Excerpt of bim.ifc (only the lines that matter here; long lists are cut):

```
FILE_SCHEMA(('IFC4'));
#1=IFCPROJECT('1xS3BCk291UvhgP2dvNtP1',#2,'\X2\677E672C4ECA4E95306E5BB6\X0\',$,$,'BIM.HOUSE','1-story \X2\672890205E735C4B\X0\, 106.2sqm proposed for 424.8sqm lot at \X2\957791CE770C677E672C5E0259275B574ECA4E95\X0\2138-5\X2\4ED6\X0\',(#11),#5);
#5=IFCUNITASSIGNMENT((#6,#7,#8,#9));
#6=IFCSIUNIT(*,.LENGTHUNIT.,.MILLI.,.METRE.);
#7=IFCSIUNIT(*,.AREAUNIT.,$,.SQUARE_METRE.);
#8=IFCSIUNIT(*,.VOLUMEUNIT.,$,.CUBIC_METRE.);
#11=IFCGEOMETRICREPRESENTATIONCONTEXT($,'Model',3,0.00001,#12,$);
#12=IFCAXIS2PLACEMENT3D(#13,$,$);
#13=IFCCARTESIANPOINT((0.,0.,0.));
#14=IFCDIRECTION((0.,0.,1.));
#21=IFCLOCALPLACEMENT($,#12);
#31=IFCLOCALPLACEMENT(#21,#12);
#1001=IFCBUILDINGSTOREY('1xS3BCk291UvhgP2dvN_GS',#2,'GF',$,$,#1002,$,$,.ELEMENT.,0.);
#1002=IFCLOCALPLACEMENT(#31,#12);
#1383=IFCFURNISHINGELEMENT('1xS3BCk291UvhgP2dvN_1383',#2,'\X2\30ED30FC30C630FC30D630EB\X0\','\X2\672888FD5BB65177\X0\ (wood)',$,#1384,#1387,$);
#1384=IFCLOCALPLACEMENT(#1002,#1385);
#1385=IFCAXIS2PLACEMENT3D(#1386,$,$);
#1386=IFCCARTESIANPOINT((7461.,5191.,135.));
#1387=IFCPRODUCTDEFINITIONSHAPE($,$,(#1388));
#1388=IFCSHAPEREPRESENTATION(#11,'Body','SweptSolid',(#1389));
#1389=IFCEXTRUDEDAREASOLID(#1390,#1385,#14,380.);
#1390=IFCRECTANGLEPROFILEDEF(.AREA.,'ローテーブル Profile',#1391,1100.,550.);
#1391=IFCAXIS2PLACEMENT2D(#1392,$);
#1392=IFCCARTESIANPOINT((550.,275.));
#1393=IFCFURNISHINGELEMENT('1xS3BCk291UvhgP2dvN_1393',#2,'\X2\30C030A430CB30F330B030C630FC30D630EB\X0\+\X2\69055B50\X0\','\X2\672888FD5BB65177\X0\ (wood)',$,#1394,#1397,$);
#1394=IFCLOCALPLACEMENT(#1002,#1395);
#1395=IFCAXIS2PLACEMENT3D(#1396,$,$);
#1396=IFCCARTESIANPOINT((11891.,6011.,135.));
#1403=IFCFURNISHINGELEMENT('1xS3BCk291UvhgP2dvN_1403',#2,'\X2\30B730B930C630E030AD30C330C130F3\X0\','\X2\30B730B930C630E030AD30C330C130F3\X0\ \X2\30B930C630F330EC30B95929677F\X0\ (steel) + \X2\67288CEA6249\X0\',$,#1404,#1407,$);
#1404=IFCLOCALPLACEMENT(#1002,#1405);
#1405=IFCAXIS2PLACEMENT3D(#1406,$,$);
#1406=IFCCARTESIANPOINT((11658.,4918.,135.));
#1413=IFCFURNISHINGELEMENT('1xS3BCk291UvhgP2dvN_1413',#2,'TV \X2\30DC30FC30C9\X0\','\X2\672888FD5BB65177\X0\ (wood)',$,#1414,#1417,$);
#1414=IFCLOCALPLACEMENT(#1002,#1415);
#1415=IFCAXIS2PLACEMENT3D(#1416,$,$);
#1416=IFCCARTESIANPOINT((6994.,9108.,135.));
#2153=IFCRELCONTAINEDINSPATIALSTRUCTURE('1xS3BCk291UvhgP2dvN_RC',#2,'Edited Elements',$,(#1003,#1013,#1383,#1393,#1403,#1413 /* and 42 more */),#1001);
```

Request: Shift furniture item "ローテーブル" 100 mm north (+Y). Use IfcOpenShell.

```python
import ifcopenshell
import ifcopenshell.api.geometry
import ifcopenshell.util.placement

model = ifcopenshell.open("bim.ifc")

item = model.by_guid("1xS3BCk291UvhgP2dvN_1383")
matrix = ifcopenshell.util.placement.get_local_placement(item.ObjectPlacement)
matrix[1, 3] += 100.0
ifcopenshell.api.geometry.edit_object_placement(model, product=item, matrix=matrix, is_si=False)

print(ifcopenshell.util.placement.get_local_placement(item.ObjectPlacement).round(3) + 0.0)

model.write("bim_v2.ifc")
```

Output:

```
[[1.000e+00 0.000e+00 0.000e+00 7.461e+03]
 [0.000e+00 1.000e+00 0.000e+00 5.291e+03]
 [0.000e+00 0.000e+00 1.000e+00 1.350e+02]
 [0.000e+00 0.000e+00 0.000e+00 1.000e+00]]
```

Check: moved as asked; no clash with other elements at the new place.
